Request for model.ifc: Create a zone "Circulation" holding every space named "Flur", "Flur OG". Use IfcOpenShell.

First a look at what the model holds.

```python
import ifcopenshell

model = ifcopenshell.open("model.ifc")
print(model.schema)
seen = {}
for space in model.by_type("IfcSpace"):
    seen[space.LongName] = seen.get(space.LongName, 0) + 1
for name, count in sorted(seen.items(), key=str):
    print(count, "x", name)
print("zones:", [z.Name for z in model.by_type("IfcZone")][:20])
```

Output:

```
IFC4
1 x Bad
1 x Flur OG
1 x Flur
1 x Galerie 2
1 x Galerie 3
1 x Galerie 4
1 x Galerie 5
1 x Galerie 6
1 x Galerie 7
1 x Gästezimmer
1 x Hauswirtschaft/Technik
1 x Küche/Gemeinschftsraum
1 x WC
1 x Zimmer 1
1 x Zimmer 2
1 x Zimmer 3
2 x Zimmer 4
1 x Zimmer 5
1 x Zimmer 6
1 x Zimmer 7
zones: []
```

```python
import ifcopenshell
import ifcopenshell.api.group
import ifcopenshell.api.root

model = ifcopenshell.open("model.ifc")

names = {"Flur", "Flur OG"}
spaces = [s for s in model.by_type("IfcSpace") if s.LongName in names]

zone = ifcopenshell.api.root.create_entity(model, ifc_class="IfcZone", name="Circulation")
ifcopenshell.api.group.assign_group(model, products=spaces, group=zone)
print(len(spaces), "spaces in", zone.Name)

model.write("model-out.ifc")
```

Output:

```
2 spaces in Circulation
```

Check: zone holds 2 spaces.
